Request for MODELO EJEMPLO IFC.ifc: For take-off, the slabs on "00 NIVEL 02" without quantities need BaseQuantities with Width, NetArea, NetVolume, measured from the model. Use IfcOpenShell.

First a look at what the model holds.

```python
import ifcopenshell
import ifcopenshell.util.element
import ifcopenshell.util.unit

model = ifcopenshell.open("MODELO EJEMPLO IFC.ifc")
print(model.schema)
for unit_type in ("LENGTHUNIT", "AREAUNIT", "VOLUMEUNIT"):
    print(unit_type, ifcopenshell.util.unit.calculate_unit_scale(model, unit_type))
storey = next(s for s in model.by_type("IfcBuildingStorey") if s.Name == "00 NIVEL 02")
slabs = [e for e in ifcopenshell.util.element.get_decomposition(storey) if e.is_a("IfcSlab")]
for e in sorted(slabs, key=lambda e: e.id()):
    print(e.id(), e.is_a(), e.Name, list(ifcopenshell.util.element.get_psets(e, qtos_only=True)), sep=" | ")
```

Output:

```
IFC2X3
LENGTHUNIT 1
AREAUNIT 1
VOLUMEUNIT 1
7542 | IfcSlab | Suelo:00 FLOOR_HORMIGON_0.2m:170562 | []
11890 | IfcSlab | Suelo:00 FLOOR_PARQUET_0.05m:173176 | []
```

```python
import ifcopenshell
import ifcopenshell.api.pset
import ifcopenshell.geom
import ifcopenshell.util.element
import ifcopenshell.util.shape
import ifcopenshell.util.unit

model = ifcopenshell.open("MODELO EJEMPLO IFC.ifc")
unit_scale = ifcopenshell.util.unit.calculate_unit_scale(model)
area_scale = ifcopenshell.util.unit.calculate_unit_scale(model, "AREAUNIT")
volume_scale = ifcopenshell.util.unit.calculate_unit_scale(model, "VOLUMEUNIT")
settings = ifcopenshell.geom.settings()

storey = next(s for s in model.by_type("IfcBuildingStorey") if s.Name == "00 NIVEL 02")
slabs = [e for e in ifcopenshell.util.element.get_decomposition(storey) if e.is_a("IfcSlab")]

for e in sorted(slabs, key=lambda e: e.id()):
    if ifcopenshell.util.element.get_psets(e, qtos_only=True, should_inherit=False):
        continue
    # Geometry comes back in metres, in the element's own axes.
    shape = ifcopenshell.geom.create_shape(settings, e)
    values = {
        "Width": ifcopenshell.util.shape.get_z(shape.geometry) / unit_scale,
        "NetArea": ifcopenshell.util.shape.get_footprint_area(shape.geometry) / area_scale,
        "NetVolume": ifcopenshell.util.shape.get_volume(shape.geometry) / volume_scale,
    }
    qto = ifcopenshell.api.pset.add_qto(model, product=e, name="BaseQuantities")
    ifcopenshell.api.pset.edit_qto(model, qto=qto, properties=values)
    print(e.id(), {k: round(v, 3) for k, v in values.items()})

model.write("MODELO EJEMPLO IFC_edited.ifc")
```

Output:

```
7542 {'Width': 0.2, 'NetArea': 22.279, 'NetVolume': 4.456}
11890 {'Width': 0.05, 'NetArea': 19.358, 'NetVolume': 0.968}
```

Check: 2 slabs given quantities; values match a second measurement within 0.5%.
